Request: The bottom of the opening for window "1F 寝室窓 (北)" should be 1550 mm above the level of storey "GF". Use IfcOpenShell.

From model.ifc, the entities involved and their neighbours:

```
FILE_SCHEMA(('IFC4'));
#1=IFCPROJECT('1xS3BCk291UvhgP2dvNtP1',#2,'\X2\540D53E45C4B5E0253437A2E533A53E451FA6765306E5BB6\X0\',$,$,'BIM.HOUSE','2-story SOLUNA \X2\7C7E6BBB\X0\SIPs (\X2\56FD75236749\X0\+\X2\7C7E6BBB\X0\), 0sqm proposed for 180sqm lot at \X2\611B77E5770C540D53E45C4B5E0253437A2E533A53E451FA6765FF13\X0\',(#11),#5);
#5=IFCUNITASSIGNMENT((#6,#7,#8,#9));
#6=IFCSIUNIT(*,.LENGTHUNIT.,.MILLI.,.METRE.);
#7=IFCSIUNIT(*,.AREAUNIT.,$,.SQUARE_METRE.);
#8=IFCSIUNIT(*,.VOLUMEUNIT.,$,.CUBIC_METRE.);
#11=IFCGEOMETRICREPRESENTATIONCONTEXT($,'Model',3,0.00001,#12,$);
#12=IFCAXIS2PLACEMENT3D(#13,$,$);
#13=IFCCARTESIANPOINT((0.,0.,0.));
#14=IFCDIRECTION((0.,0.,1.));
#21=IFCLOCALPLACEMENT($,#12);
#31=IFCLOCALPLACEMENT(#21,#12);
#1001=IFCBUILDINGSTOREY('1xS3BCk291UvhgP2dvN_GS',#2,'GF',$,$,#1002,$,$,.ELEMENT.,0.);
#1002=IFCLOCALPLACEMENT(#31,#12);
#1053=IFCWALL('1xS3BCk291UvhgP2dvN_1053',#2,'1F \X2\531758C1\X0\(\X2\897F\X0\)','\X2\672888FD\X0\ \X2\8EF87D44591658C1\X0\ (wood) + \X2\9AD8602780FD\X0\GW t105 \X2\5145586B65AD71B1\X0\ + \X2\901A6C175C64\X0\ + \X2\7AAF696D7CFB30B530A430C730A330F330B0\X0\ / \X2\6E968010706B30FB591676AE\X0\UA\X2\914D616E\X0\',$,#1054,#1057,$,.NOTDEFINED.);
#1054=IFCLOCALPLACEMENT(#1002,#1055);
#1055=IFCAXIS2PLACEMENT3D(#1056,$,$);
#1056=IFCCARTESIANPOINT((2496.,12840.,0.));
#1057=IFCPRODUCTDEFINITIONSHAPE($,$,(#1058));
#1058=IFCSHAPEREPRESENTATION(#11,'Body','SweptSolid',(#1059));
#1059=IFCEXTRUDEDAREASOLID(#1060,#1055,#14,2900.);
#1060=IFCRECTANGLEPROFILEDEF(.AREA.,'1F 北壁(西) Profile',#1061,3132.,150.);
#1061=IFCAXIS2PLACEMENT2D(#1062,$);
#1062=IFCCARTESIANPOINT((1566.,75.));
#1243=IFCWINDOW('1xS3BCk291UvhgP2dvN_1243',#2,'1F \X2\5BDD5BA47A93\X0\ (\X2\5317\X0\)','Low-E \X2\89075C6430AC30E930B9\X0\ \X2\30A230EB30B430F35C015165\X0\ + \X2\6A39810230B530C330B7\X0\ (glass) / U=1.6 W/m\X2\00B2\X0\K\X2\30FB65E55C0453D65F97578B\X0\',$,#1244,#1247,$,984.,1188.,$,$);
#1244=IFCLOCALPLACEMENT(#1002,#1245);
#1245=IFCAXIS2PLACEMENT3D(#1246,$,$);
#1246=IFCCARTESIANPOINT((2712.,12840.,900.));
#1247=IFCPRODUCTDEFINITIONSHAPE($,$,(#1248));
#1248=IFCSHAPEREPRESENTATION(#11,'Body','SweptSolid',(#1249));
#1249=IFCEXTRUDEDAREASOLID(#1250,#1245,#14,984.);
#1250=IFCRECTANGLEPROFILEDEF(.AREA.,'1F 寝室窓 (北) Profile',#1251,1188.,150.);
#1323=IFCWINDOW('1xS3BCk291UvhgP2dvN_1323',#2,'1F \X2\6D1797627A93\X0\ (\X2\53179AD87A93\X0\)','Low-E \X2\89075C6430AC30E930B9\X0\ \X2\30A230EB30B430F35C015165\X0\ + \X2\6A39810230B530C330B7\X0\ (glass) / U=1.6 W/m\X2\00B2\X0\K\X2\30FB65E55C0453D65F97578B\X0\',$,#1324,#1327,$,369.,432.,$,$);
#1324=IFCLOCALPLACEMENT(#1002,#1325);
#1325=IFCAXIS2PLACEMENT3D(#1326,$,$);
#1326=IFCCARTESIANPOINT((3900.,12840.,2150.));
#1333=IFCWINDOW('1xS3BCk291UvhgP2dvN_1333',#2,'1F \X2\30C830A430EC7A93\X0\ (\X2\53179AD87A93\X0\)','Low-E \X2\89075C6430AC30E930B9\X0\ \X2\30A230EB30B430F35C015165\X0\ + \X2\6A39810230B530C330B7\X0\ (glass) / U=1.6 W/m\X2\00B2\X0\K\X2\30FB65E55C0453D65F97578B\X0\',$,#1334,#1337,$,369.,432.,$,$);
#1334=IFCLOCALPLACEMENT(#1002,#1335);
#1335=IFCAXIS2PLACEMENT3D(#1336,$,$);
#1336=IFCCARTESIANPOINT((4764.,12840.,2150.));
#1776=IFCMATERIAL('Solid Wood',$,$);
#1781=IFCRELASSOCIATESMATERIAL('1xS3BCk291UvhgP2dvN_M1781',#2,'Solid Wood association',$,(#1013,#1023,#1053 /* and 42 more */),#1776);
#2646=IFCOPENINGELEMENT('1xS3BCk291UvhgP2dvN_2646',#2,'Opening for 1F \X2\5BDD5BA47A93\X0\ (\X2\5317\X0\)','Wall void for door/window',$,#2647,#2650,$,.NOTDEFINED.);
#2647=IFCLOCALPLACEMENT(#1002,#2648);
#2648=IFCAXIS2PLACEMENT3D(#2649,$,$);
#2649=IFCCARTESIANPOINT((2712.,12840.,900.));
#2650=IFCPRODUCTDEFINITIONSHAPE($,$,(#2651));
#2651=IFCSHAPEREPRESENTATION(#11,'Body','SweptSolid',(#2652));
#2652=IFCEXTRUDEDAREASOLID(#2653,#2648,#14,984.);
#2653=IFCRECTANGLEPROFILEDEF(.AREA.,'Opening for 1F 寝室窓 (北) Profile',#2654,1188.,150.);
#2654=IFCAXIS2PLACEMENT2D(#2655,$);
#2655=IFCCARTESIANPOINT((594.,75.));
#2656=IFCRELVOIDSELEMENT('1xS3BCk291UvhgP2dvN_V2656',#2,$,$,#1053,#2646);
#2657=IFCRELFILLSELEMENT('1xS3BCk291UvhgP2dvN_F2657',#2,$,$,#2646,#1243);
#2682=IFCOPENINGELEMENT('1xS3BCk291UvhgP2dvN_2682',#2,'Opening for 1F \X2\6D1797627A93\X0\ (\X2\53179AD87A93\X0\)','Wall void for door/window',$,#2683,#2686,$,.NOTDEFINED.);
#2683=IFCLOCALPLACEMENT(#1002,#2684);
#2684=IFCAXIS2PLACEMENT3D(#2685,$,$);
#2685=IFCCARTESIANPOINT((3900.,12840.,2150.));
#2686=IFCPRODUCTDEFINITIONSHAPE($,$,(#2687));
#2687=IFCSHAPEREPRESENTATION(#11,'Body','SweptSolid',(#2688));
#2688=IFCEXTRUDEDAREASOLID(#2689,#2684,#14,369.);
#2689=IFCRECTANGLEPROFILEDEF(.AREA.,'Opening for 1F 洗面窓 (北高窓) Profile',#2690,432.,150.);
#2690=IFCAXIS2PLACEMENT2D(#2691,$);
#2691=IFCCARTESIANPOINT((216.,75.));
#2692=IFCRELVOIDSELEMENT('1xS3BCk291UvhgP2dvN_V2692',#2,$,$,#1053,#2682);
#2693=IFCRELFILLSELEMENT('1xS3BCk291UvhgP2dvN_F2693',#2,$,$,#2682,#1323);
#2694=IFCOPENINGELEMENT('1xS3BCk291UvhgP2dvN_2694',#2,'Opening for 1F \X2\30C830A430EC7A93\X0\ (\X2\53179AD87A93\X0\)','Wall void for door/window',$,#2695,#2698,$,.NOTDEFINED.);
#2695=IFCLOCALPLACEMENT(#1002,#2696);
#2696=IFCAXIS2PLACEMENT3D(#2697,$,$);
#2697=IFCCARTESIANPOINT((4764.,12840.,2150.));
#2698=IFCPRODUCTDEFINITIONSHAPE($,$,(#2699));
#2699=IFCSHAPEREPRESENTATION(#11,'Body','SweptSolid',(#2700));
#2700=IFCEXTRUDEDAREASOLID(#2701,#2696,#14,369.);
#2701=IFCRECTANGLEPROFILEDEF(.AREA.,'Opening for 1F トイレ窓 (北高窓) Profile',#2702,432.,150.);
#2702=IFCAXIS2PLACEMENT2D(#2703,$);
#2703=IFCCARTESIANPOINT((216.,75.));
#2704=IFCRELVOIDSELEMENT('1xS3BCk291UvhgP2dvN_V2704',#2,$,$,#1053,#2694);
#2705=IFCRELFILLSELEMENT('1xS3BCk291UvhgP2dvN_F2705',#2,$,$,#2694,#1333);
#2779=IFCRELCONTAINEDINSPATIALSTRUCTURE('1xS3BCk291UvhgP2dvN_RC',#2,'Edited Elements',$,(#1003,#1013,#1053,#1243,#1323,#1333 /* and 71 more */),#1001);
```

```python
import numpy as np
import ifcopenshell
import ifcopenshell.api.geometry
import ifcopenshell.geom
import ifcopenshell.util.element
import ifcopenshell.util.placement
import ifcopenshell.util.shape
import ifcopenshell.util.unit

model = ifcopenshell.open("model.ifc")
unit_scale = ifcopenshell.util.unit.calculate_unit_scale(model)

window = model.by_id(1243)
opening = window.FillsVoids[0].RelatingOpeningElement
storey = ifcopenshell.util.element.get_container(window, ifc_class="IfcBuildingStorey")
level = ifcopenshell.util.placement.get_local_placement(storey.ObjectPlacement)[2, 3]

# The opening's origin need not be at the sill, so measure its lowest point.
shape = ifcopenshell.geom.create_shape(ifcopenshell.geom.settings(), opening)
bottom = ifcopenshell.util.shape.get_shape_bottom_elevation(shape, shape.geometry) / unit_scale
dz = level + 1.55 / unit_scale - bottom

shift = np.array([0.0, 0.0, dz])
# The window is not placed relative to its opening, so move both.
for product in (opening, window):
    matrix = ifcopenshell.util.placement.get_local_placement(product.ObjectPlacement)
    matrix[:3, 3] += shift
    ifcopenshell.api.geometry.edit_object_placement(model, product=product, matrix=matrix, is_si=False)

print(f"moved by {dz * unit_scale:+.3f} m")

model.write("model_updated.ifc")
```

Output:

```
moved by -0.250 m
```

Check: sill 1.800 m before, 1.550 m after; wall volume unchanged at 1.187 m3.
